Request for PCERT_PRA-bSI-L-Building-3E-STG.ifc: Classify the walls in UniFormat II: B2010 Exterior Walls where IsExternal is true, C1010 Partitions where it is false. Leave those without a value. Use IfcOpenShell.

First a look at what the model holds.

```python
import ifcopenshell
import ifcopenshell.util.element

model = ifcopenshell.open("PCERT_PRA-bSI-L-Building-3E-STG.ifc")
print(model.schema)
print("classifications:", [c.Name for c in model.by_type("IfcClassification")])
values = [ifcopenshell.util.element.get_pset(e, "Pset_WallCommon", "IsExternal") for e in model.by_type("IfcWall")]
for value in (True, False, None):
    print("IsExternal", value, values.count(value))
```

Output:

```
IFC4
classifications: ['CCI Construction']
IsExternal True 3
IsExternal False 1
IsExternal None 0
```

```python
import ifcopenshell
import ifcopenshell.api.classification
import ifcopenshell.util.element

model = ifcopenshell.open("PCERT_PRA-bSI-L-Building-3E-STG.ifc")

system = ifcopenshell.api.classification.add_classification(model, classification="UniFormat II")

walls = model.by_type("IfcWall")
external = {e: ifcopenshell.util.element.get_pset(e, "Pset_WallCommon", "IsExternal") for e in walls}
for flag, code, name in ((True, "B2010", "Exterior Walls"), (False, "C1010", "Partitions")):
    products = [e for e in walls if external[e] is flag]
    ifcopenshell.api.classification.add_reference(
        model, products=products, classification=system, identification=code, name=name
    )
    print(code, len(products))

model.write("PCERT_PRA-bSI-L-Building-3E-STG-out.ifc")
```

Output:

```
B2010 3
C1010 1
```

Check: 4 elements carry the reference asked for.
